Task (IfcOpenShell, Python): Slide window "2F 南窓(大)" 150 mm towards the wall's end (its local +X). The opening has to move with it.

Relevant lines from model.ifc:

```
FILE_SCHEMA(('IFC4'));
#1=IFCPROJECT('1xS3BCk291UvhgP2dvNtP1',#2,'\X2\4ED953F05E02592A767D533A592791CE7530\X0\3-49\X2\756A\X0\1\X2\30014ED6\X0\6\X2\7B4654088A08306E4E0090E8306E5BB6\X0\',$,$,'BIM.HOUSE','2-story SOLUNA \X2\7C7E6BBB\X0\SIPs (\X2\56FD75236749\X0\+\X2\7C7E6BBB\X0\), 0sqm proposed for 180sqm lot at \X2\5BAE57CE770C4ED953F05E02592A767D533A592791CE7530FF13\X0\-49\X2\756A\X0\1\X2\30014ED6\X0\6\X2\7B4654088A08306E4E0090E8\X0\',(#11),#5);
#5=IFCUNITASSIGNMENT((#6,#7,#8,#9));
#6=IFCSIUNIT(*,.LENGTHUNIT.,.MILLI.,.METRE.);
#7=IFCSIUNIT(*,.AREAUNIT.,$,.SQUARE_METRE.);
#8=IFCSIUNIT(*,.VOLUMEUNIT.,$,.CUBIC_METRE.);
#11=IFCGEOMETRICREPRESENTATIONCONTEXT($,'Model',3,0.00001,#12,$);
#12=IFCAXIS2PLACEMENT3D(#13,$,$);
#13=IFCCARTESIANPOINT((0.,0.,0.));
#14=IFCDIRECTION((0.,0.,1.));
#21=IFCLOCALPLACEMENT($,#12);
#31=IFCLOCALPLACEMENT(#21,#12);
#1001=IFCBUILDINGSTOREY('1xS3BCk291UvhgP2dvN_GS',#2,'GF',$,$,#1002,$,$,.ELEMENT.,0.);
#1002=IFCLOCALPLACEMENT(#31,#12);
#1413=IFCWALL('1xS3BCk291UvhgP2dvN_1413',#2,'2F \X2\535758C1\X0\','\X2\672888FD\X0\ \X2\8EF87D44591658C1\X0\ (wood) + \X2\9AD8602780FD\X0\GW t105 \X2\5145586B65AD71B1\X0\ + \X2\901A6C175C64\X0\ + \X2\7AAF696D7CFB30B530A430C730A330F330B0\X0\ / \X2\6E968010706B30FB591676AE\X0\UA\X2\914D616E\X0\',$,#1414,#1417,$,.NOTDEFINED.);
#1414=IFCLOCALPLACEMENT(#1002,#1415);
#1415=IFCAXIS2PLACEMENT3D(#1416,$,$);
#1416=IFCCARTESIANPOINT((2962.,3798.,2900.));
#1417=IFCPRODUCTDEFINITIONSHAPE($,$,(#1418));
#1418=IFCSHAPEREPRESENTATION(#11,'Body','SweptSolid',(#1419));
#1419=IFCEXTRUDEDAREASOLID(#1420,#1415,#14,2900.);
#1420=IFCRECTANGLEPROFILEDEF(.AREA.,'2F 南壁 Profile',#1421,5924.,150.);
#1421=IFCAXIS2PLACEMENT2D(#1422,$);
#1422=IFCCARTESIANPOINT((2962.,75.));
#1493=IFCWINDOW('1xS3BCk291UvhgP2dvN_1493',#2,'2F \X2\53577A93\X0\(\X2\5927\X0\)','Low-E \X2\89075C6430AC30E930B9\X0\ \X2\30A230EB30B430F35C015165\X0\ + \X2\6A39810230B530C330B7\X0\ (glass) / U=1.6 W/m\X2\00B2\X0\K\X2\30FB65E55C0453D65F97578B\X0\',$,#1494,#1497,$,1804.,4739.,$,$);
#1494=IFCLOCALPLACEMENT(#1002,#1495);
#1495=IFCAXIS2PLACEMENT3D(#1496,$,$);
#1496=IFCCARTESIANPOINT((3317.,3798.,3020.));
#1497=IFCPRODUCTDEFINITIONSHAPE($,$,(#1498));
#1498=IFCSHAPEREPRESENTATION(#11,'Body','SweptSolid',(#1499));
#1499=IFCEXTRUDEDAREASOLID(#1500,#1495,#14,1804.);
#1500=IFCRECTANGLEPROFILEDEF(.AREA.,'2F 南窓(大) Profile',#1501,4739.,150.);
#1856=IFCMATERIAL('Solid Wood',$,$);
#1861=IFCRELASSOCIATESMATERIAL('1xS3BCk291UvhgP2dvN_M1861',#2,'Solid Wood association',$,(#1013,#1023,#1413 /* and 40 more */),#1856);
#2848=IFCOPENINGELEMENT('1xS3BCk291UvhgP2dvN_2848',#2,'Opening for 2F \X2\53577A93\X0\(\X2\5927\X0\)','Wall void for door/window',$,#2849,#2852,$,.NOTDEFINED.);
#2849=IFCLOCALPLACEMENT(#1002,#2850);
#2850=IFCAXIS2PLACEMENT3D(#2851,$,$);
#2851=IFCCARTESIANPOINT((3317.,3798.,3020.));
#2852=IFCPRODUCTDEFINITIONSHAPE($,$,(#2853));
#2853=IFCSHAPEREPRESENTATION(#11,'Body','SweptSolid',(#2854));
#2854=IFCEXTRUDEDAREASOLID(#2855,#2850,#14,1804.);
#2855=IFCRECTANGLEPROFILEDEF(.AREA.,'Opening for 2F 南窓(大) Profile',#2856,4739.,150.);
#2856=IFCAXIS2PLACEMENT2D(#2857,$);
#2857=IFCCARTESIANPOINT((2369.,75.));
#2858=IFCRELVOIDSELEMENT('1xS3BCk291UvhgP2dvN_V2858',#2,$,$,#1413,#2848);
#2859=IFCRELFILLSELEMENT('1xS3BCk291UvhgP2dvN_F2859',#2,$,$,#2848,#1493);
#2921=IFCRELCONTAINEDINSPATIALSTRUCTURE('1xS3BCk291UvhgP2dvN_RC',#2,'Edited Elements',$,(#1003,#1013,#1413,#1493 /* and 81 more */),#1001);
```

```python
import ifcopenshell
import ifcopenshell.api.geometry
import ifcopenshell.util.placement
import ifcopenshell.util.unit

model = ifcopenshell.open("model.ifc")
unit_scale = ifcopenshell.util.unit.calculate_unit_scale(model)

window = model.by_id(1493)
opening = window.FillsVoids[0].RelatingOpeningElement
wall = opening.VoidsElements[0].RelatingBuildingElement

wall_matrix = ifcopenshell.util.placement.get_local_placement(wall.ObjectPlacement)
shift = wall_matrix[:3, 0] * 0.15 / unit_scale
before = ifcopenshell.util.placement.get_local_placement(window.ObjectPlacement)[:3, 3].copy()

# The window is not placed relative to its opening, so move both.
for product in (opening, window):
    matrix = ifcopenshell.util.placement.get_local_placement(product.ObjectPlacement)
    matrix[:3, 3] += shift
    ifcopenshell.api.geometry.edit_object_placement(model, product=product, matrix=matrix, is_si=False)

after = ifcopenshell.util.placement.get_local_placement(window.ObjectPlacement)[:3, 3]
print("window moved by", (after - before).round(3) + 0.0)

model.write("model_updated.ifc")
```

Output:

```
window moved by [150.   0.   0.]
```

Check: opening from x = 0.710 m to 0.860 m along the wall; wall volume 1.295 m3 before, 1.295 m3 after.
